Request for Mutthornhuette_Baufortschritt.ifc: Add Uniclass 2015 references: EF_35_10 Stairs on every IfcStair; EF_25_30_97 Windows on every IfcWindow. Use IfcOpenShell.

First a look at what the model holds.

```python
import ifcopenshell

model = ifcopenshell.open("Mutthornhuette_Baufortschritt.ifc")
print(model.schema)
print("classifications:", [c.Name for c in model.by_type("IfcClassification")])
for ifc_class in ("IfcDoor", "IfcRoof", "IfcStair", "IfcWall", "IfcWindow"):
    print(ifc_class, len(model.by_type(ifc_class)))
```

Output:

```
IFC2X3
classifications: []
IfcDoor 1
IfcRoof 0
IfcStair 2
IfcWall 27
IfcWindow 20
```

```python
import ifcopenshell
import ifcopenshell.api.classification

model = ifcopenshell.open("Mutthornhuette_Baufortschritt.ifc")

# IFC2X3 requires Source and Edition and has no link from the project to the system.
system = model.create_entity("IfcClassification", Source="NBS", Edition="2015", Name="Uniclass 2015")

codes = {
    "IfcStair": ("EF_35_10", "Stairs"),
    "IfcWindow": ("EF_25_30_97", "Windows"),
}
for ifc_class, (code, name) in codes.items():
    products = model.by_type(ifc_class)
    ifcopenshell.api.classification.add_reference(
        model, products=products, classification=system, identification=code, name=name
    )
    print(code, len(products))

model.write("Mutthornhuette_Baufortschritt_v2.ifc")
```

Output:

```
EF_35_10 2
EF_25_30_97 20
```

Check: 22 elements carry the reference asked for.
